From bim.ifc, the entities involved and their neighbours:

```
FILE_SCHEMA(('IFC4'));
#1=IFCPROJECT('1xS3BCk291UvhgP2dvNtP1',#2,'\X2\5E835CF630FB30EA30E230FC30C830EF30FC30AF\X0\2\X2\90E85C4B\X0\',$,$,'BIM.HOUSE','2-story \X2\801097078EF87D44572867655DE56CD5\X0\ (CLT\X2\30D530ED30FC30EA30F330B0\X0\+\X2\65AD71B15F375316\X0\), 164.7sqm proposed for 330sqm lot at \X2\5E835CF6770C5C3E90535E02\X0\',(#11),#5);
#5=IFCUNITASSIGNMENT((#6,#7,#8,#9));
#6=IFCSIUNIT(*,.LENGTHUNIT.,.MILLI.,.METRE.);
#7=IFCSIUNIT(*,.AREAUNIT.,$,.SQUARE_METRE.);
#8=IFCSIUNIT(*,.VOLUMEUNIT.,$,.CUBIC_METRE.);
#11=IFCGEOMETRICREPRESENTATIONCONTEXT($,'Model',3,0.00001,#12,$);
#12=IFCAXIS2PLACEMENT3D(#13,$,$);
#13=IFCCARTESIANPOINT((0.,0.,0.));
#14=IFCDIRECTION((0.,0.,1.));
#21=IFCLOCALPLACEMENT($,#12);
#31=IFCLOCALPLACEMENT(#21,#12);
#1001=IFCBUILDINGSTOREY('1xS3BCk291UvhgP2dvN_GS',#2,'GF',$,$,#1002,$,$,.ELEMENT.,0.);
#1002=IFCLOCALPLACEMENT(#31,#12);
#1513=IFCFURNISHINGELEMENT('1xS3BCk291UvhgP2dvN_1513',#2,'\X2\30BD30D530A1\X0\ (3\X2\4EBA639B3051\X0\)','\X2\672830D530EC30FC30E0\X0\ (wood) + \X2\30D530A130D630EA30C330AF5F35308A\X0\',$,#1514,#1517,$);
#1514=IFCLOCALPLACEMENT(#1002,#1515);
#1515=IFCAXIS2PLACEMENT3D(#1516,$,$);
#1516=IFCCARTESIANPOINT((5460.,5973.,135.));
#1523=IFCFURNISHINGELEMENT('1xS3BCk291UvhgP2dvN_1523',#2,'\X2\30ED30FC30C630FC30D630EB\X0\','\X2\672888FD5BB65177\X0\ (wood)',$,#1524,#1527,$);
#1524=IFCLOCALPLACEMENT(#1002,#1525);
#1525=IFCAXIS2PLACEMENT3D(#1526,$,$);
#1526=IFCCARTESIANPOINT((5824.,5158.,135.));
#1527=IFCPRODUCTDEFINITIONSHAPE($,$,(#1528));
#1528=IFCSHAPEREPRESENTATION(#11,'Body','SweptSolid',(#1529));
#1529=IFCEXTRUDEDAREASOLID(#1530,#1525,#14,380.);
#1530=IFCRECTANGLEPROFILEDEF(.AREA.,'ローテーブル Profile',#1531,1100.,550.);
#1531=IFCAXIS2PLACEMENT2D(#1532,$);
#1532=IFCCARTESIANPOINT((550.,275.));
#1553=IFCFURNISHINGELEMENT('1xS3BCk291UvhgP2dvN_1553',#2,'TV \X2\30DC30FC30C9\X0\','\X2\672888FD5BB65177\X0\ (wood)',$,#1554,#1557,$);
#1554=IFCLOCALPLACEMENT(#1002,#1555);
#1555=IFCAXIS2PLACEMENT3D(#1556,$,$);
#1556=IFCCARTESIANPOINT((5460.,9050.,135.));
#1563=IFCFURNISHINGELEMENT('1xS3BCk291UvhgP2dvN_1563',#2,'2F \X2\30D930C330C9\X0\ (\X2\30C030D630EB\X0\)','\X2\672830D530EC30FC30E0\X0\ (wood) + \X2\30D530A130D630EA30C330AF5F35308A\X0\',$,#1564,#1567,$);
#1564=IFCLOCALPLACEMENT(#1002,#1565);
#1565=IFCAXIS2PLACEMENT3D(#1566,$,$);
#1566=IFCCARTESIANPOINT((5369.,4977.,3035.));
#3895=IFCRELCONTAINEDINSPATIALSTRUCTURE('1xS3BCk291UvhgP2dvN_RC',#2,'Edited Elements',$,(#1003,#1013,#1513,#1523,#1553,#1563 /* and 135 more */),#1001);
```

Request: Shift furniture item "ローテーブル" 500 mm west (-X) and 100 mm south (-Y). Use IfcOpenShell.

```python
import ifcopenshell
import ifcopenshell.api.geometry
import ifcopenshell.util.placement

model = ifcopenshell.open("bim.ifc")

item = model.by_id(1523)
matrix = ifcopenshell.util.placement.get_local_placement(item.ObjectPlacement)
matrix[0, 3] -= 500.0
matrix[1, 3] -= 100.0
ifcopenshell.api.geometry.edit_object_placement(model, product=item, matrix=matrix, is_si=False)

print(ifcopenshell.util.placement.get_local_placement(item.ObjectPlacement).round(3) + 0.0)

model.write("bim_edited.ifc")
```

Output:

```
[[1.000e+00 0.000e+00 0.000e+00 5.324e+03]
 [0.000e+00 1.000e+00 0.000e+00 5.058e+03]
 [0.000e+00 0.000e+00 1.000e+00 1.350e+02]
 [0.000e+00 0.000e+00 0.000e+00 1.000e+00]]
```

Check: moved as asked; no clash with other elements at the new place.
